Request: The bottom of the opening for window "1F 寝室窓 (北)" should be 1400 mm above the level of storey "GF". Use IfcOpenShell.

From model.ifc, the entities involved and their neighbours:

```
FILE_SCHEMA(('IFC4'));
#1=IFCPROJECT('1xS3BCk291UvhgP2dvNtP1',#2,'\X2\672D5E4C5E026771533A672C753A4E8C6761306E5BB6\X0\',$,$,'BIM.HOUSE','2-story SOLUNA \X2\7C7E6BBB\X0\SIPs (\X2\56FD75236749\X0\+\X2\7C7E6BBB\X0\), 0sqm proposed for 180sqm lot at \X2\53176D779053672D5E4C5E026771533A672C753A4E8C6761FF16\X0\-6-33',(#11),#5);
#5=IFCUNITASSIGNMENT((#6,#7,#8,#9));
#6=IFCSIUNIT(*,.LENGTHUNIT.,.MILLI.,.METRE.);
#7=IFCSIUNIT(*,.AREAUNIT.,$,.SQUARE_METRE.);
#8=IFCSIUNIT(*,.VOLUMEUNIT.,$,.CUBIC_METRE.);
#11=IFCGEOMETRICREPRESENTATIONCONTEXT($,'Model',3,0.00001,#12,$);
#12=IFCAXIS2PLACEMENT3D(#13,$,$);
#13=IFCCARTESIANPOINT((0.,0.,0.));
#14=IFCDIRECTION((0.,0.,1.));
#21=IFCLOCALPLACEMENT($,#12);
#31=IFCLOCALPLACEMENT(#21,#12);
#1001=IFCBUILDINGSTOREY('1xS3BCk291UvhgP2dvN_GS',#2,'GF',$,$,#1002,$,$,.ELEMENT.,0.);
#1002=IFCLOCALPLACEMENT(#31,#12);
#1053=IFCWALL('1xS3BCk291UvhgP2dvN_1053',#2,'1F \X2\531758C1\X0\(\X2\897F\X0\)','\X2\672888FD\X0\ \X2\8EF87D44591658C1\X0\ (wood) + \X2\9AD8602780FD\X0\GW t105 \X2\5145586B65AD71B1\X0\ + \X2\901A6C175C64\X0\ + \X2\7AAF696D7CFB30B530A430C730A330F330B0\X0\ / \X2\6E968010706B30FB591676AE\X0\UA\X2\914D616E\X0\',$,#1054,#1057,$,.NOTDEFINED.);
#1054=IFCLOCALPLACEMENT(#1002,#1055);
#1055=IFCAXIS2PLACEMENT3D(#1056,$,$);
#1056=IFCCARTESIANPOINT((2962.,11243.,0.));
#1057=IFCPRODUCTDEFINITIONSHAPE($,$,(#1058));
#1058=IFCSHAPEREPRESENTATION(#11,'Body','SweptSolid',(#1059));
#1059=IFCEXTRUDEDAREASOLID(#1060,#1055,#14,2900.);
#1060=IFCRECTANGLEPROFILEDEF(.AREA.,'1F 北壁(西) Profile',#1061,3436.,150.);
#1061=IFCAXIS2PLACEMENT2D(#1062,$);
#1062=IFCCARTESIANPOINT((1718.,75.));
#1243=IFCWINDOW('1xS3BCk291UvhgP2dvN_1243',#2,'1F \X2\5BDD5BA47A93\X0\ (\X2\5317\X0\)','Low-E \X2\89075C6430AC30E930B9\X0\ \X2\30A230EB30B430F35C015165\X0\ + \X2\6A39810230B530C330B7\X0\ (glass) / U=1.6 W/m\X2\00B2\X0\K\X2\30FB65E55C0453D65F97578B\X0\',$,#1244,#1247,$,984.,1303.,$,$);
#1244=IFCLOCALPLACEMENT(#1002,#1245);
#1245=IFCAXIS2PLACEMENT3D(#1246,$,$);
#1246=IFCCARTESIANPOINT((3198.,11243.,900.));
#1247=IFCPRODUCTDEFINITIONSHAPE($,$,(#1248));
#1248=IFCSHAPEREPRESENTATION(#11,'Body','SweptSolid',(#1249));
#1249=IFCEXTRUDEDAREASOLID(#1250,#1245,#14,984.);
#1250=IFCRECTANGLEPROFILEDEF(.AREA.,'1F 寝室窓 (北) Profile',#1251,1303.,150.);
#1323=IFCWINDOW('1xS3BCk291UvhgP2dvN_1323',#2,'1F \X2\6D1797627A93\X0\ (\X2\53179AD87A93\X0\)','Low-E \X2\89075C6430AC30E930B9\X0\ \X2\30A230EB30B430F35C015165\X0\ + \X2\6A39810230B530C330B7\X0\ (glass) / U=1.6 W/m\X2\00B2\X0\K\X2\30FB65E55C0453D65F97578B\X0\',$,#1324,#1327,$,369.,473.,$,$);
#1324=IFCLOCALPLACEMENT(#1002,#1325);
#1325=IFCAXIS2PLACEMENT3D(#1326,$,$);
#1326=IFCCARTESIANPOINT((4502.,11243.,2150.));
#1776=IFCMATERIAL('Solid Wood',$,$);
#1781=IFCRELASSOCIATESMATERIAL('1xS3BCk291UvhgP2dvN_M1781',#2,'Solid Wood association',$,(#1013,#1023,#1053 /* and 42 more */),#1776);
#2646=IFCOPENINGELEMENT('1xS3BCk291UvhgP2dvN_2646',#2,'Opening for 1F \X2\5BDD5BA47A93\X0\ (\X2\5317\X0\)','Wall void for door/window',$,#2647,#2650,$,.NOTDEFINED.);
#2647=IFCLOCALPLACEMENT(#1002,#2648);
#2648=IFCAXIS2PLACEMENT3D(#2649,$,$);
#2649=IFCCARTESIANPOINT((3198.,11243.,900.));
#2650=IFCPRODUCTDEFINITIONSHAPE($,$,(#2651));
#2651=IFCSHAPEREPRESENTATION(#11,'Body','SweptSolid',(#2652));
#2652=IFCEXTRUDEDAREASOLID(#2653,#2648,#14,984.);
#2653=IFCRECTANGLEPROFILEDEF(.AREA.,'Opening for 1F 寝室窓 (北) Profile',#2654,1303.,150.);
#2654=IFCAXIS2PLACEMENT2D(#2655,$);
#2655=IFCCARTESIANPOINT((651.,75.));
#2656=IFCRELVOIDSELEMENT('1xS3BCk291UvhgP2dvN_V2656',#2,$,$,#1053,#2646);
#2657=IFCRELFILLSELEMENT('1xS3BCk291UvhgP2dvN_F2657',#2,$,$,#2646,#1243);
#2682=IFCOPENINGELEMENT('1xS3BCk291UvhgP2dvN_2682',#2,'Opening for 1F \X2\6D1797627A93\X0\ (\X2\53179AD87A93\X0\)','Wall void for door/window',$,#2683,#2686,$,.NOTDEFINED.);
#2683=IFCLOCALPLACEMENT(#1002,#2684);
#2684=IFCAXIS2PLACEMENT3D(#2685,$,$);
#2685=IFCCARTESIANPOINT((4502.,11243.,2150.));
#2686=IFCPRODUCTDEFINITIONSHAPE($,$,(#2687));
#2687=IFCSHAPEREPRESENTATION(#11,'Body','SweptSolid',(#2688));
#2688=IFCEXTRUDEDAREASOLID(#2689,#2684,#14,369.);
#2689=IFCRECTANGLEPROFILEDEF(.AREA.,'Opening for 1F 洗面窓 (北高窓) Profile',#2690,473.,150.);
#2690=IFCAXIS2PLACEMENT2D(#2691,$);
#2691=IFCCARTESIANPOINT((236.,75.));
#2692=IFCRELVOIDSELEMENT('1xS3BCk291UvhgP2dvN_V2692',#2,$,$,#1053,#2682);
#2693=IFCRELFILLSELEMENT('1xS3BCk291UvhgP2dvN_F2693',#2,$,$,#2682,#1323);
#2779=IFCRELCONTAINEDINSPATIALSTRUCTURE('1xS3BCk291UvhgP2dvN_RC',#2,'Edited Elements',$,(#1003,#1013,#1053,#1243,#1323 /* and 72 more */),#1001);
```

```python
import numpy as np
import ifcopenshell
import ifcopenshell.api.geometry
import ifcopenshell.geom
import ifcopenshell.util.element
import ifcopenshell.util.placement
import ifcopenshell.util.shape
import ifcopenshell.util.unit

model = ifcopenshell.open("model.ifc")
unit_scale = ifcopenshell.util.unit.calculate_unit_scale(model)

window = model.by_guid("1xS3BCk291UvhgP2dvN_1243")
opening = window.FillsVoids[0].RelatingOpeningElement
storey = ifcopenshell.util.element.get_container(window, ifc_class="IfcBuildingStorey")
level = ifcopenshell.util.placement.get_local_placement(storey.ObjectPlacement)[2, 3]

# The opening's origin need not be at the sill, so measure its lowest point.
shape = ifcopenshell.geom.create_shape(ifcopenshell.geom.settings(), opening)
bottom = ifcopenshell.util.shape.get_shape_bottom_elevation(shape, shape.geometry) / unit_scale
dz = level + 1.4 / unit_scale - bottom

shift = np.array([0.0, 0.0, dz])
# The window is not placed relative to its opening, so move both.
for product in (opening, window):
    matrix = ifcopenshell.util.placement.get_local_placement(product.ObjectPlacement)
    matrix[:3, 3] += shift
    ifcopenshell.api.geometry.edit_object_placement(model, product=product, matrix=matrix, is_si=False)

print(f"moved by {dz * unit_scale:+.3f} m")

model.write("model_updated.ifc")
```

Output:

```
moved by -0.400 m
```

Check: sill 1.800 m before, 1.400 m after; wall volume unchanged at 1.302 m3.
